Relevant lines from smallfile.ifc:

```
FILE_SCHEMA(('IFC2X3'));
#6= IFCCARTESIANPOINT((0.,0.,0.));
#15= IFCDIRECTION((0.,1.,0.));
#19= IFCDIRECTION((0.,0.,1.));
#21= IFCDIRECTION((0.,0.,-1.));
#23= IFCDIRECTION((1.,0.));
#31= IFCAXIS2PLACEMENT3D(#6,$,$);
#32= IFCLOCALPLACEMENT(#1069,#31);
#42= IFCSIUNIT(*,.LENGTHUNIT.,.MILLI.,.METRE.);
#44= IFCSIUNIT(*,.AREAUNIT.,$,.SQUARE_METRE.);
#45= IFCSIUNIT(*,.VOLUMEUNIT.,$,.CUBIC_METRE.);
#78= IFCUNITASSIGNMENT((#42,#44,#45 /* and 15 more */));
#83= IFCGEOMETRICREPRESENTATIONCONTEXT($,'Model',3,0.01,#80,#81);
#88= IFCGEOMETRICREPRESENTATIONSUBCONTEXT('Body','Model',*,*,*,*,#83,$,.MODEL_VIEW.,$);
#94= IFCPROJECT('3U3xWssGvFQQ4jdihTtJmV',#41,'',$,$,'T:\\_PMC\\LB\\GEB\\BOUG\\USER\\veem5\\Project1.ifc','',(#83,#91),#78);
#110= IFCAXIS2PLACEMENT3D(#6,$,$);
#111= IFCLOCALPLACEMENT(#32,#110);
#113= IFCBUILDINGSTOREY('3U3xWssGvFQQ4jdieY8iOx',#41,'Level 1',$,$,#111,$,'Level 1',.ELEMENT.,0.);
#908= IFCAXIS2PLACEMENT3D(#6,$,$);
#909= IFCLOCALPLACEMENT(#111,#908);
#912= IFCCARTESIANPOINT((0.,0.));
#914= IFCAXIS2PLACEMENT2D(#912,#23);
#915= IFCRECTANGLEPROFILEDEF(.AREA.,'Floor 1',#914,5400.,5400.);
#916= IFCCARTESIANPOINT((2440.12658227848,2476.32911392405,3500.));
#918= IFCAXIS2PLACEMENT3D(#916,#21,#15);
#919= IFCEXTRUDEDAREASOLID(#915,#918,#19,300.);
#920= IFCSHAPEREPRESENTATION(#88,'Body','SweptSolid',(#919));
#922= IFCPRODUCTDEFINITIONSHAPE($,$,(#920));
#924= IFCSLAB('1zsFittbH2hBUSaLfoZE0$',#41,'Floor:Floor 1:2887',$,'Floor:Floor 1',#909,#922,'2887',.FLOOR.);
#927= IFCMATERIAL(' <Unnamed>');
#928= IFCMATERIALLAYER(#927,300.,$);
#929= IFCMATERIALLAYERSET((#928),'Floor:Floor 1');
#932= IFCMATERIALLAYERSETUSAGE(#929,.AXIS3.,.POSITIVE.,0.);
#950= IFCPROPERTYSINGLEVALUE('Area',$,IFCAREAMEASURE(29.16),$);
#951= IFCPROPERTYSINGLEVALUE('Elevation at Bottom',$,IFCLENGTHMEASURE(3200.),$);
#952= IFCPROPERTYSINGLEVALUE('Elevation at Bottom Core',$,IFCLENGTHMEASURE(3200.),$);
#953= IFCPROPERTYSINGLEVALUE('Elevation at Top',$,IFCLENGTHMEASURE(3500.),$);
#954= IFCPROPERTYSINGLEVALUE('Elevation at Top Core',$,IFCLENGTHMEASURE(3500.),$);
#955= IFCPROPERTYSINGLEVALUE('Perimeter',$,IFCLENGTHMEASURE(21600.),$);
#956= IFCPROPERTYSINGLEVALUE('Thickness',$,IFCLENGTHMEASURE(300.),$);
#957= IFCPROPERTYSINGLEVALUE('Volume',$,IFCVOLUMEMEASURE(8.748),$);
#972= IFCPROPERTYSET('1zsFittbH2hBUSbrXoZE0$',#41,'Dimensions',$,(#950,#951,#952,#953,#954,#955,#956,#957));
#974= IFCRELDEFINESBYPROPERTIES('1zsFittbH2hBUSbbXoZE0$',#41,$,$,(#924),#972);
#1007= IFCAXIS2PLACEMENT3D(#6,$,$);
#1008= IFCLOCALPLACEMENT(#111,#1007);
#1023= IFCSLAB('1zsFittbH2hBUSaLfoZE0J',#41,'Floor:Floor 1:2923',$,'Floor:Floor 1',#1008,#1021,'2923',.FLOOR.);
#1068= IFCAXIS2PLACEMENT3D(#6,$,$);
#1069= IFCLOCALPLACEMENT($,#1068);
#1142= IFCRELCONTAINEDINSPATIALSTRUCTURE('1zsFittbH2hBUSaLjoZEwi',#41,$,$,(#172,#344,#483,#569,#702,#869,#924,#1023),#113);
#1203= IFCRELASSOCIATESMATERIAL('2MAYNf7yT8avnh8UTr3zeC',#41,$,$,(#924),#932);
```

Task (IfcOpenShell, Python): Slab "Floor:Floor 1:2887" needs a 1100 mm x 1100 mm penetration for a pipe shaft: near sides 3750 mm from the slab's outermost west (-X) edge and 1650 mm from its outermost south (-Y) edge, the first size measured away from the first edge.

```python
import numpy as np
import ifcopenshell
import ifcopenshell.api.feature
import ifcopenshell.api.geometry
import ifcopenshell.api.pset
import ifcopenshell.api.root
import ifcopenshell.geom
import ifcopenshell.util.element
import ifcopenshell.util.placement
import ifcopenshell.util.representation
import ifcopenshell.util.shape
import ifcopenshell.util.unit

model = ifcopenshell.open("smallfile.ifc")
unit_scale = ifcopenshell.util.unit.calculate_unit_scale(model)
area_scale = ifcopenshell.util.unit.calculate_unit_scale(model, "AREAUNIT")
volume_scale = ifcopenshell.util.unit.calculate_unit_scale(model, "VOLUMEUNIT")
settings = ifcopenshell.geom.settings()


def volume(element):
    """Net volume in cubic metres, openings subtracted."""
    shape = ifcopenshell.geom.create_shape(settings, element)
    return ifcopenshell.util.shape.get_volume(shape.geometry)


slab = model.by_id(924)
before = volume(slab)

# Extent in the slab's own axes, in metres. The edges named are its -X and -Y sides.
slab_shape = ifcopenshell.geom.create_shape(settings, slab)
vertices = ifcopenshell.util.shape.get_vertices(slab_shape.geometry)
x_min, y_min, bottom = vertices.min(axis=0)
top = vertices[:, 2].max()

opening = ifcopenshell.api.root.create_entity(model, ifc_class="IfcOpeningElement", name="Pipe shaft opening")
context = ifcopenshell.util.representation.get_context(model, "Model", "Body", "MODEL_VIEW")
width, depth = 1.1, 1.1
outline = [(0.0, 0.0), (width, 0.0), (width, depth), (0.0, depth), (0.0, 0.0)]
# Overshoot both faces by 50 mm so the cut is clean.
shape = ifcopenshell.api.geometry.add_slab_representation(
    model, context=context, depth=top - bottom + 0.1, polyline=outline
)
ifcopenshell.api.geometry.assign_representation(model, product=opening, representation=shape)

matrix = ifcopenshell.util.placement.get_local_placement(slab.ObjectPlacement)
matrix[:, 3] = matrix @ np.append(np.array([x_min + 3.75, y_min + 1.65, bottom - 0.05]) / unit_scale, 1.0)
ifcopenshell.api.geometry.edit_object_placement(model, product=opening, matrix=matrix, is_si=False)
ifcopenshell.api.feature.add_feature(model, feature=opening, element=slab)

after = volume(slab)

# Update the slab's stored quantities.
pset = model.by_id(ifcopenshell.util.element.get_pset(slab, "Dimensions", should_inherit=False)["id"])
ifcopenshell.api.pset.edit_pset(model, pset=pset, properties={
    "Area": model.create_entity("IfcAreaMeasure", after / (top - bottom) / area_scale),
    "Volume": model.create_entity("IfcVolumeMeasure", after / volume_scale),
})

print(f"slab volume {before:.3f} -> {after:.3f} m3")

model.write("smallfile_v2.ifc")
```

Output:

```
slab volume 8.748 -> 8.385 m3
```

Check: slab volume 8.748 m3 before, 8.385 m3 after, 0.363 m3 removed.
